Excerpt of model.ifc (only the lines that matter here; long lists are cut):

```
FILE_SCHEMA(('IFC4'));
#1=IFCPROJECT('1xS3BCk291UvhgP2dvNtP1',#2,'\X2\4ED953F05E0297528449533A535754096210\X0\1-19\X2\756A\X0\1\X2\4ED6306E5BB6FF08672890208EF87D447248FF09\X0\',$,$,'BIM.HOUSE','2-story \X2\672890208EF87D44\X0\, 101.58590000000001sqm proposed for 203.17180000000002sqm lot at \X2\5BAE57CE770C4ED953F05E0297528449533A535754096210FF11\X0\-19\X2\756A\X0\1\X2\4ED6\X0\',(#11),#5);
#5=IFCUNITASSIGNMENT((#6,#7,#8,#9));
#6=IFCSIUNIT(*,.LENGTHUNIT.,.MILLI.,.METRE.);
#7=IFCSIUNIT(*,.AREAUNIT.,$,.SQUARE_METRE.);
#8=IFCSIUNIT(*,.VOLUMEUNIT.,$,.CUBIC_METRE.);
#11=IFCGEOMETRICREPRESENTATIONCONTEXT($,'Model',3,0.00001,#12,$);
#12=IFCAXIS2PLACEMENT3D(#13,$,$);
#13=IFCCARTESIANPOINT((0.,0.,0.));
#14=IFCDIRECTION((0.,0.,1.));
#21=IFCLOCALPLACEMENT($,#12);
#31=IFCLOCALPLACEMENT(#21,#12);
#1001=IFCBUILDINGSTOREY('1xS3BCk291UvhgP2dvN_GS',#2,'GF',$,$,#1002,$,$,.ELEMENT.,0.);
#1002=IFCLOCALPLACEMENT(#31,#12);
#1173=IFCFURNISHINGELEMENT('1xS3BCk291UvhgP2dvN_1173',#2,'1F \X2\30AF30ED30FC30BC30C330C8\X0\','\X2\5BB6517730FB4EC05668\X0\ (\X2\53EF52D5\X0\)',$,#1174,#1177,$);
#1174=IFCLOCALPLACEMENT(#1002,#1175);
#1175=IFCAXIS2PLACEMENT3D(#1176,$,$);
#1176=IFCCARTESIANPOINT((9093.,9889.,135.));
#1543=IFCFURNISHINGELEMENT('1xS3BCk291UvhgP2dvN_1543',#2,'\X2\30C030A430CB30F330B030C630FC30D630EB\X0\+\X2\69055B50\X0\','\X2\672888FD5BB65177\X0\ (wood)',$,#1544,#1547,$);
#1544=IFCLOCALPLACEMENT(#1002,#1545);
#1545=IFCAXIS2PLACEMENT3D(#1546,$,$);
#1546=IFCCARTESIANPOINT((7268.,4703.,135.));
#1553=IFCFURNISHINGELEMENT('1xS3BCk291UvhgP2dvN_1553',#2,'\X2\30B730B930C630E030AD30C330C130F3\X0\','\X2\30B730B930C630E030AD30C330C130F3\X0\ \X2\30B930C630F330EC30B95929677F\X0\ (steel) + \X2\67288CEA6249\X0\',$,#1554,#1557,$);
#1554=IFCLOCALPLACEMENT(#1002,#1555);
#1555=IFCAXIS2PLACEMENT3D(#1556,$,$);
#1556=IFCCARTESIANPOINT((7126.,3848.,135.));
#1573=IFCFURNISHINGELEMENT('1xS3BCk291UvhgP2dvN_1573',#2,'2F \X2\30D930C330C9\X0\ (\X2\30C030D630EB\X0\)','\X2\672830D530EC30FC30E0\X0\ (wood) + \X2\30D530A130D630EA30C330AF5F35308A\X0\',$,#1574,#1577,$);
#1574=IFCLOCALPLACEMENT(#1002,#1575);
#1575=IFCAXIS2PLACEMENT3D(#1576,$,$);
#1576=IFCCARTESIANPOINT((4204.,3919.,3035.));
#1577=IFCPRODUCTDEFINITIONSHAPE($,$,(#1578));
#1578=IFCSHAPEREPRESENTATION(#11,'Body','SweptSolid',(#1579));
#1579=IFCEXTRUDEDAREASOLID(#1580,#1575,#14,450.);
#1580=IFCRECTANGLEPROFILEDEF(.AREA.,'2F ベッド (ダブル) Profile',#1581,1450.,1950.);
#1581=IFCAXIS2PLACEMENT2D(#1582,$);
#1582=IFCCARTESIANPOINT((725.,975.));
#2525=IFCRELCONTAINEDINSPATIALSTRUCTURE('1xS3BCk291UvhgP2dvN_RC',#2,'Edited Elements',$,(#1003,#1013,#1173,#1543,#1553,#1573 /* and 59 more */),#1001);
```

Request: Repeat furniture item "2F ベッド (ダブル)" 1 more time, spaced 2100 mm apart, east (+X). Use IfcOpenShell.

```python
import numpy as np
import ifcopenshell
import ifcopenshell.api.geometry
import ifcopenshell.api.root
import ifcopenshell.util.element
import ifcopenshell.util.placement
import ifcopenshell.util.unit

model = ifcopenshell.open("model.ifc")
unit_scale = ifcopenshell.util.unit.calculate_unit_scale(model)


def reuse_history(source, copy):
    """copy_class also copies each property set's owner history, people and application; keep the originals."""
    for rel in copy.IsDefinedBy:
        if rel.is_a("IfcRelDefinesByProperties") and (history := rel.RelatingPropertyDefinition.OwnerHistory):
            rel.RelatingPropertyDefinition.OwnerHistory = source.OwnerHistory
            ifcopenshell.util.element.remove_deep2(model, history)


source = model.by_id(1573)
base = ifcopenshell.util.placement.get_local_placement(source.ObjectPlacement)
step = np.array([1.0, 0.0, 0.0]) * 2.1 / unit_scale

for i in range(1, 2):
    copy = ifcopenshell.api.root.copy_class(model, product=source)
    copy.Representation = ifcopenshell.util.element.copy_deep(
        model, source.Representation, exclude=["IfcGeometricRepresentationContext", "IfcRepresentationMap"]
    )
    reuse_history(source, copy)
    matrix = base.copy()
    matrix[:3, 3] += i * step
    print("added at", matrix[:3, 3].round(3) + 0.0)
    ifcopenshell.api.geometry.edit_object_placement(model, product=copy, matrix=matrix, is_si=False)

model.write("model_rev.ifc")
```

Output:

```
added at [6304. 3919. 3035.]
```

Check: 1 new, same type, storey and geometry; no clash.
